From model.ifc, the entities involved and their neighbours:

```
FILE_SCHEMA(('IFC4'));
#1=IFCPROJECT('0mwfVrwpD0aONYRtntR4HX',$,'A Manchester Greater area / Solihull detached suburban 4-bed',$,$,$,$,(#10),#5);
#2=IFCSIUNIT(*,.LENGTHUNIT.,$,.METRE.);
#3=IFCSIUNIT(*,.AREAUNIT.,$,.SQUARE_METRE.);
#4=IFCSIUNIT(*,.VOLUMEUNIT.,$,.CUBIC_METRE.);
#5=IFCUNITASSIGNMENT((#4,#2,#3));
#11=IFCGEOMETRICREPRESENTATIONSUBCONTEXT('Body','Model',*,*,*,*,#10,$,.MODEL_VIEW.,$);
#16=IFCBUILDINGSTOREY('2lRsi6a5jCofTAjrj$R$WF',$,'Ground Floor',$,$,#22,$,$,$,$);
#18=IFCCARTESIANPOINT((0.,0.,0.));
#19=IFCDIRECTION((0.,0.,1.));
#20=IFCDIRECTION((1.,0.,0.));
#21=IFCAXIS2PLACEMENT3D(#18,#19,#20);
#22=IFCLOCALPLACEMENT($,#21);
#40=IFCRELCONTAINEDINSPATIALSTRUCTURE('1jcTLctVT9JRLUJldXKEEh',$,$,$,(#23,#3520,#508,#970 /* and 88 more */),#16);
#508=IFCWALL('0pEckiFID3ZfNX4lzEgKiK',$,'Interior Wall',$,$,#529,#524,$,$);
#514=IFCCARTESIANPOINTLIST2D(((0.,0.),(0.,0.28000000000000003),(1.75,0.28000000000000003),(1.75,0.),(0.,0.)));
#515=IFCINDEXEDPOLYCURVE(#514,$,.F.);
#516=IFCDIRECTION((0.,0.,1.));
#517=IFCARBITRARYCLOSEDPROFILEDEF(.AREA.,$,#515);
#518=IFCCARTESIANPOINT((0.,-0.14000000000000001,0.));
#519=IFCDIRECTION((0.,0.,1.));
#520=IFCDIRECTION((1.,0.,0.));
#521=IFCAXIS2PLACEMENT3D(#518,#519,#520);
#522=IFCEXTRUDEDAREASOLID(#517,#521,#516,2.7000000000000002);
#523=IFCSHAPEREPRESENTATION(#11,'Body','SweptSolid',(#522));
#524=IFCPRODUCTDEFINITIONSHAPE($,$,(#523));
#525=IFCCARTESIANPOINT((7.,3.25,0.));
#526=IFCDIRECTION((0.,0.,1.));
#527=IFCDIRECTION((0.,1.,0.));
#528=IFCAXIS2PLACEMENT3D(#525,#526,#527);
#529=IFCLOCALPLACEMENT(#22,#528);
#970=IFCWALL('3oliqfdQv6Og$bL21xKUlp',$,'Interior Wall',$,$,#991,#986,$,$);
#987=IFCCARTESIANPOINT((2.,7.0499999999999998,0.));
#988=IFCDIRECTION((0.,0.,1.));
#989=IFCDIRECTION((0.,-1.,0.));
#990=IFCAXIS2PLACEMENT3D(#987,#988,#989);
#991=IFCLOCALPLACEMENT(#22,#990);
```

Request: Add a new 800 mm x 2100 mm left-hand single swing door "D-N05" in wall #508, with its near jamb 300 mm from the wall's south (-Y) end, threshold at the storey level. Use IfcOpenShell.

```python
import numpy as np
import ifcopenshell
import ifcopenshell.api.feature
import ifcopenshell.api.geometry
import ifcopenshell.api.root
import ifcopenshell.api.spatial
import ifcopenshell.geom
import ifcopenshell.util.element
import ifcopenshell.util.placement
import ifcopenshell.util.representation
import ifcopenshell.util.shape
import ifcopenshell.util.unit

model = ifcopenshell.open("model.ifc")
unit_scale = ifcopenshell.util.unit.calculate_unit_scale(model)
settings = ifcopenshell.geom.settings()


def volume(element):
    """Net volume in cubic metres, openings subtracted."""
    shape = ifcopenshell.geom.create_shape(settings, element)
    return ifcopenshell.util.shape.get_volume(shape.geometry)


wall = model.by_guid("0pEckiFID3ZfNX4lzEgKiK")
storey = ifcopenshell.util.element.get_container(wall, ifc_class="IfcBuildingStorey")
context = ifcopenshell.util.representation.get_context(model, "Model", "Body", "MODEL_VIEW")
before = volume(wall)

width, height, from_end, sill = 0.8, 2.1, 0.3, 0.0  # metres

# The wall runs along its own X axis, and the end named is its -X end.
wall_shape = ifcopenshell.geom.create_shape(settings, wall)
x, y, z = ifcopenshell.util.shape.get_vertices(wall_shape.geometry).T
start = x.min() + from_end
face, thickness = float(y.min()), float(y.max() - y.min())
wall_matrix = ifcopenshell.util.placement.get_local_placement(wall.ObjectPlacement)
level = ifcopenshell.util.placement.get_local_placement(storey.ObjectPlacement)[2, 3]


def in_wall(x, y):
    """Placement at x, y metres in the wall's axes, at sill height."""
    matrix = wall_matrix.copy()
    matrix[:, 3] = wall_matrix @ np.array([x / unit_scale, y / unit_scale, 0.0, 1.0])
    matrix[2, 3] = level + sill / unit_scale
    return matrix


# Opening: a box that overshoots both wall faces by 50 mm.
opening = ifcopenshell.api.root.create_entity(model, ifc_class="IfcOpeningElement", predefined_type="OPENING")
box = ifcopenshell.api.geometry.add_wall_representation(
    model, context=context, length=width, height=height, thickness=thickness + 0.1
)
ifcopenshell.api.geometry.assign_representation(model, product=opening, representation=box)
ifcopenshell.api.geometry.edit_object_placement(model, product=opening, matrix=in_wall(start, face - 0.05), is_si=False)
ifcopenshell.api.feature.add_feature(model, feature=opening, element=wall)

door = ifcopenshell.api.root.create_entity(model, ifc_class="IfcDoor", name="D-N05", predefined_type="DOOR")
door.OverallWidth, door.OverallHeight = width / unit_scale, height / unit_scale
door.OperationType = "SINGLE_SWING_LEFT"
body = ifcopenshell.api.geometry.add_door_representation(
    model,
    context=context,
    overall_width=door.OverallWidth,
    overall_height=door.OverallHeight,
    operation_type="SINGLE_SWING_LEFT",
    lining_properties={"LiningDepth": thickness / unit_scale, "ThresholdDepth": thickness / unit_scale},
)
ifcopenshell.api.geometry.assign_representation(model, product=door, representation=body)
ifcopenshell.api.spatial.assign_container(model, products=[door], relating_structure=storey)
ifcopenshell.api.feature.add_filling(model, opening=opening, element=door)

# The lining spans the wall, so the door starts at the wall face.
ifcopenshell.api.geometry.edit_object_placement(model, product=door, matrix=in_wall(start, face), is_si=False)

after = volume(wall)

print(f"wall volume {before:.3f} -> {after:.3f} m3")

model.write("model_edited.ifc")
```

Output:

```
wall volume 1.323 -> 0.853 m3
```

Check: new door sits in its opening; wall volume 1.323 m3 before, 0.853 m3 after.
